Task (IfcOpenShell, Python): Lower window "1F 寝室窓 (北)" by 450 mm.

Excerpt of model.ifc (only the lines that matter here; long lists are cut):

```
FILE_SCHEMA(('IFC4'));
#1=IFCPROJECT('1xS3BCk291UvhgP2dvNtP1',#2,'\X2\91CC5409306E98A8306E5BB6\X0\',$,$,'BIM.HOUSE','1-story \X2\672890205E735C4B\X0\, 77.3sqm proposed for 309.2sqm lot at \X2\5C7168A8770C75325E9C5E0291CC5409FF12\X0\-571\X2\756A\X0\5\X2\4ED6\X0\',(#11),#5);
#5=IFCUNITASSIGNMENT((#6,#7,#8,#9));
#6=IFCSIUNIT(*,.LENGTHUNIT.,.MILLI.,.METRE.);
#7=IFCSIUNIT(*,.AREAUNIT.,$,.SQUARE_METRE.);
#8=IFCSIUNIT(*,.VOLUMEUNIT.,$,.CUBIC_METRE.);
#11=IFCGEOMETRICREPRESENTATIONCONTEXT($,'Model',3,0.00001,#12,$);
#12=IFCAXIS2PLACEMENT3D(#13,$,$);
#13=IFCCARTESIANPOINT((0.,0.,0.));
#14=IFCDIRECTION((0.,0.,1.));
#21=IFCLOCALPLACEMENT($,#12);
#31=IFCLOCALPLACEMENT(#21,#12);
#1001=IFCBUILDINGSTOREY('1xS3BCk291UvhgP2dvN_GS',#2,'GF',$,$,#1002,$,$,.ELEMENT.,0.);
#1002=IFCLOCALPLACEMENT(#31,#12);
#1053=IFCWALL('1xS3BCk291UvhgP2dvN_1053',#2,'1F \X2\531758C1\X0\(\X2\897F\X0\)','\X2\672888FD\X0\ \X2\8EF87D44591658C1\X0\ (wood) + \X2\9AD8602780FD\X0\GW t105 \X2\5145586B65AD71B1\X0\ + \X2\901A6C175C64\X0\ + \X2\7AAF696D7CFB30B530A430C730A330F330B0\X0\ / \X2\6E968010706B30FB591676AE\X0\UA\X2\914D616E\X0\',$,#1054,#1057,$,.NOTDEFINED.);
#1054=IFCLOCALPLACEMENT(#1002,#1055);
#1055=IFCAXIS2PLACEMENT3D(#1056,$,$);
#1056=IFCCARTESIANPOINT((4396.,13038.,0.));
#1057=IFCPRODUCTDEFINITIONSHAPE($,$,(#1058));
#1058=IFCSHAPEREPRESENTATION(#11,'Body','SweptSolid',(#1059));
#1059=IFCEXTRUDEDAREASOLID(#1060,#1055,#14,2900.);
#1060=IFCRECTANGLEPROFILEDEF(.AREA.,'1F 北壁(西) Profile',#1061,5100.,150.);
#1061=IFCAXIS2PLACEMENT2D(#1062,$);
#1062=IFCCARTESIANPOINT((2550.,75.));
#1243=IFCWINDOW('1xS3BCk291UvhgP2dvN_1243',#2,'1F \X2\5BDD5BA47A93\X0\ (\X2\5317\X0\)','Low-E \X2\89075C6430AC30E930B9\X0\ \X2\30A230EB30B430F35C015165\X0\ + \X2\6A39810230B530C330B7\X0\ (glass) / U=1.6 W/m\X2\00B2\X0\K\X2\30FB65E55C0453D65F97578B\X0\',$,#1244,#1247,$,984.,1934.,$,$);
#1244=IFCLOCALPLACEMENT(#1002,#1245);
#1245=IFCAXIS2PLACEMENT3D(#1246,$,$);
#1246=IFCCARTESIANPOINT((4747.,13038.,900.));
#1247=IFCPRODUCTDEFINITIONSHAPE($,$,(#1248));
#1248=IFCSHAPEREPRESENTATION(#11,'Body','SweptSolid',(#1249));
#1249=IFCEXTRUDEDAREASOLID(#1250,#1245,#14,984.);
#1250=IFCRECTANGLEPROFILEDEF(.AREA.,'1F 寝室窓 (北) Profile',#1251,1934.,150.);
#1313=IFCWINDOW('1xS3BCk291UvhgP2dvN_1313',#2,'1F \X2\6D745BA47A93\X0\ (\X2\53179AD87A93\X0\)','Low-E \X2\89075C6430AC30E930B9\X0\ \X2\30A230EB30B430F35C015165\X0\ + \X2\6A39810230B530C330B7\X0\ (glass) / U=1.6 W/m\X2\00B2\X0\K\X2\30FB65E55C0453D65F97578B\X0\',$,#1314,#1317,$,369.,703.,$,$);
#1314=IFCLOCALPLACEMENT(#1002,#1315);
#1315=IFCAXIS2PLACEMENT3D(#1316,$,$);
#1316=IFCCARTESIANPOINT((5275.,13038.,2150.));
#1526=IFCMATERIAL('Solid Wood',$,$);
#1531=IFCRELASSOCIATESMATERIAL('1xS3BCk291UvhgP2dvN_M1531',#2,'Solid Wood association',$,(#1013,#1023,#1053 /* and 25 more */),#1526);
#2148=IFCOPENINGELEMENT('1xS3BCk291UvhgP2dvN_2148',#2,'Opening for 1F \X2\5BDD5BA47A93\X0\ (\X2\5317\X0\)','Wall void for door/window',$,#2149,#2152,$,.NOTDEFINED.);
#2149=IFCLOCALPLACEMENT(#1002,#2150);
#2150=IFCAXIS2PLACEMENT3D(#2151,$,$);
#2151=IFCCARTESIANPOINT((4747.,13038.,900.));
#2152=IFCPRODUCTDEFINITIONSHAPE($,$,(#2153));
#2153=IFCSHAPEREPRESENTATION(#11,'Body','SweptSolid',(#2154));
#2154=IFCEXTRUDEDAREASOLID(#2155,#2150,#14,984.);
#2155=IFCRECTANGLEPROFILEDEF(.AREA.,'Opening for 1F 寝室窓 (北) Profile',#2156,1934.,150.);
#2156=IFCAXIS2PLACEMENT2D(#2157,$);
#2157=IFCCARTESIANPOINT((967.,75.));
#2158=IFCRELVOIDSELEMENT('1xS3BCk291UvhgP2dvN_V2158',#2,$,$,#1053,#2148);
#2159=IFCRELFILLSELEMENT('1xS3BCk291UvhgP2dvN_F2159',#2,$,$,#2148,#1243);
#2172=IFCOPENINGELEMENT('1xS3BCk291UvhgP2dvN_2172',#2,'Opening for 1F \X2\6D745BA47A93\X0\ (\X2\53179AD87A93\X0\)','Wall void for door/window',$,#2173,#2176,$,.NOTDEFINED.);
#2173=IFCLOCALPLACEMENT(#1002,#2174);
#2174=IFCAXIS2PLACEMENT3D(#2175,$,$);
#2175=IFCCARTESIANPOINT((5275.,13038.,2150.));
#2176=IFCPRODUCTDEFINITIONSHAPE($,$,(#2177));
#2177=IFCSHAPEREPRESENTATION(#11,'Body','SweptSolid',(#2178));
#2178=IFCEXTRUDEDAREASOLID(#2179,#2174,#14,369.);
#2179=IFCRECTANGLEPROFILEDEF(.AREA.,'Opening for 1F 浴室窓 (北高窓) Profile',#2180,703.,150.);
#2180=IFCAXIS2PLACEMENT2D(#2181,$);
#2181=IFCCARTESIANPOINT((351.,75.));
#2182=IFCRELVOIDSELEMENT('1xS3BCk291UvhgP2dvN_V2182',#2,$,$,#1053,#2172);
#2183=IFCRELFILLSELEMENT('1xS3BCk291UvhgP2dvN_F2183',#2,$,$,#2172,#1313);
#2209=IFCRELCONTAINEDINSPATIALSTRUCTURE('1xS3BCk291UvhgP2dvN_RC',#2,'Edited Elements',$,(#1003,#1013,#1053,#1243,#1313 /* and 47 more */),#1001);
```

```python
import numpy as np
import ifcopenshell
import ifcopenshell.api.geometry
import ifcopenshell.util.placement
import ifcopenshell.util.unit

model = ifcopenshell.open("model.ifc")
unit_scale = ifcopenshell.util.unit.calculate_unit_scale(model)

window = model.by_guid("1xS3BCk291UvhgP2dvN_1243")
opening = window.FillsVoids[0].RelatingOpeningElement
dz = -450.0

shift = np.array([0.0, 0.0, dz])
# The window is not placed relative to its opening, so move both.
for product in (opening, window):
    matrix = ifcopenshell.util.placement.get_local_placement(product.ObjectPlacement)
    matrix[:3, 3] += shift
    ifcopenshell.api.geometry.edit_object_placement(model, product=product, matrix=matrix, is_si=False)

print(f"moved by {dz * unit_scale:+.3f} m")

model.write("model_v2.ifc")
```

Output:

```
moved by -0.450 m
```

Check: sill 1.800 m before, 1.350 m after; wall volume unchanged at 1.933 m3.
